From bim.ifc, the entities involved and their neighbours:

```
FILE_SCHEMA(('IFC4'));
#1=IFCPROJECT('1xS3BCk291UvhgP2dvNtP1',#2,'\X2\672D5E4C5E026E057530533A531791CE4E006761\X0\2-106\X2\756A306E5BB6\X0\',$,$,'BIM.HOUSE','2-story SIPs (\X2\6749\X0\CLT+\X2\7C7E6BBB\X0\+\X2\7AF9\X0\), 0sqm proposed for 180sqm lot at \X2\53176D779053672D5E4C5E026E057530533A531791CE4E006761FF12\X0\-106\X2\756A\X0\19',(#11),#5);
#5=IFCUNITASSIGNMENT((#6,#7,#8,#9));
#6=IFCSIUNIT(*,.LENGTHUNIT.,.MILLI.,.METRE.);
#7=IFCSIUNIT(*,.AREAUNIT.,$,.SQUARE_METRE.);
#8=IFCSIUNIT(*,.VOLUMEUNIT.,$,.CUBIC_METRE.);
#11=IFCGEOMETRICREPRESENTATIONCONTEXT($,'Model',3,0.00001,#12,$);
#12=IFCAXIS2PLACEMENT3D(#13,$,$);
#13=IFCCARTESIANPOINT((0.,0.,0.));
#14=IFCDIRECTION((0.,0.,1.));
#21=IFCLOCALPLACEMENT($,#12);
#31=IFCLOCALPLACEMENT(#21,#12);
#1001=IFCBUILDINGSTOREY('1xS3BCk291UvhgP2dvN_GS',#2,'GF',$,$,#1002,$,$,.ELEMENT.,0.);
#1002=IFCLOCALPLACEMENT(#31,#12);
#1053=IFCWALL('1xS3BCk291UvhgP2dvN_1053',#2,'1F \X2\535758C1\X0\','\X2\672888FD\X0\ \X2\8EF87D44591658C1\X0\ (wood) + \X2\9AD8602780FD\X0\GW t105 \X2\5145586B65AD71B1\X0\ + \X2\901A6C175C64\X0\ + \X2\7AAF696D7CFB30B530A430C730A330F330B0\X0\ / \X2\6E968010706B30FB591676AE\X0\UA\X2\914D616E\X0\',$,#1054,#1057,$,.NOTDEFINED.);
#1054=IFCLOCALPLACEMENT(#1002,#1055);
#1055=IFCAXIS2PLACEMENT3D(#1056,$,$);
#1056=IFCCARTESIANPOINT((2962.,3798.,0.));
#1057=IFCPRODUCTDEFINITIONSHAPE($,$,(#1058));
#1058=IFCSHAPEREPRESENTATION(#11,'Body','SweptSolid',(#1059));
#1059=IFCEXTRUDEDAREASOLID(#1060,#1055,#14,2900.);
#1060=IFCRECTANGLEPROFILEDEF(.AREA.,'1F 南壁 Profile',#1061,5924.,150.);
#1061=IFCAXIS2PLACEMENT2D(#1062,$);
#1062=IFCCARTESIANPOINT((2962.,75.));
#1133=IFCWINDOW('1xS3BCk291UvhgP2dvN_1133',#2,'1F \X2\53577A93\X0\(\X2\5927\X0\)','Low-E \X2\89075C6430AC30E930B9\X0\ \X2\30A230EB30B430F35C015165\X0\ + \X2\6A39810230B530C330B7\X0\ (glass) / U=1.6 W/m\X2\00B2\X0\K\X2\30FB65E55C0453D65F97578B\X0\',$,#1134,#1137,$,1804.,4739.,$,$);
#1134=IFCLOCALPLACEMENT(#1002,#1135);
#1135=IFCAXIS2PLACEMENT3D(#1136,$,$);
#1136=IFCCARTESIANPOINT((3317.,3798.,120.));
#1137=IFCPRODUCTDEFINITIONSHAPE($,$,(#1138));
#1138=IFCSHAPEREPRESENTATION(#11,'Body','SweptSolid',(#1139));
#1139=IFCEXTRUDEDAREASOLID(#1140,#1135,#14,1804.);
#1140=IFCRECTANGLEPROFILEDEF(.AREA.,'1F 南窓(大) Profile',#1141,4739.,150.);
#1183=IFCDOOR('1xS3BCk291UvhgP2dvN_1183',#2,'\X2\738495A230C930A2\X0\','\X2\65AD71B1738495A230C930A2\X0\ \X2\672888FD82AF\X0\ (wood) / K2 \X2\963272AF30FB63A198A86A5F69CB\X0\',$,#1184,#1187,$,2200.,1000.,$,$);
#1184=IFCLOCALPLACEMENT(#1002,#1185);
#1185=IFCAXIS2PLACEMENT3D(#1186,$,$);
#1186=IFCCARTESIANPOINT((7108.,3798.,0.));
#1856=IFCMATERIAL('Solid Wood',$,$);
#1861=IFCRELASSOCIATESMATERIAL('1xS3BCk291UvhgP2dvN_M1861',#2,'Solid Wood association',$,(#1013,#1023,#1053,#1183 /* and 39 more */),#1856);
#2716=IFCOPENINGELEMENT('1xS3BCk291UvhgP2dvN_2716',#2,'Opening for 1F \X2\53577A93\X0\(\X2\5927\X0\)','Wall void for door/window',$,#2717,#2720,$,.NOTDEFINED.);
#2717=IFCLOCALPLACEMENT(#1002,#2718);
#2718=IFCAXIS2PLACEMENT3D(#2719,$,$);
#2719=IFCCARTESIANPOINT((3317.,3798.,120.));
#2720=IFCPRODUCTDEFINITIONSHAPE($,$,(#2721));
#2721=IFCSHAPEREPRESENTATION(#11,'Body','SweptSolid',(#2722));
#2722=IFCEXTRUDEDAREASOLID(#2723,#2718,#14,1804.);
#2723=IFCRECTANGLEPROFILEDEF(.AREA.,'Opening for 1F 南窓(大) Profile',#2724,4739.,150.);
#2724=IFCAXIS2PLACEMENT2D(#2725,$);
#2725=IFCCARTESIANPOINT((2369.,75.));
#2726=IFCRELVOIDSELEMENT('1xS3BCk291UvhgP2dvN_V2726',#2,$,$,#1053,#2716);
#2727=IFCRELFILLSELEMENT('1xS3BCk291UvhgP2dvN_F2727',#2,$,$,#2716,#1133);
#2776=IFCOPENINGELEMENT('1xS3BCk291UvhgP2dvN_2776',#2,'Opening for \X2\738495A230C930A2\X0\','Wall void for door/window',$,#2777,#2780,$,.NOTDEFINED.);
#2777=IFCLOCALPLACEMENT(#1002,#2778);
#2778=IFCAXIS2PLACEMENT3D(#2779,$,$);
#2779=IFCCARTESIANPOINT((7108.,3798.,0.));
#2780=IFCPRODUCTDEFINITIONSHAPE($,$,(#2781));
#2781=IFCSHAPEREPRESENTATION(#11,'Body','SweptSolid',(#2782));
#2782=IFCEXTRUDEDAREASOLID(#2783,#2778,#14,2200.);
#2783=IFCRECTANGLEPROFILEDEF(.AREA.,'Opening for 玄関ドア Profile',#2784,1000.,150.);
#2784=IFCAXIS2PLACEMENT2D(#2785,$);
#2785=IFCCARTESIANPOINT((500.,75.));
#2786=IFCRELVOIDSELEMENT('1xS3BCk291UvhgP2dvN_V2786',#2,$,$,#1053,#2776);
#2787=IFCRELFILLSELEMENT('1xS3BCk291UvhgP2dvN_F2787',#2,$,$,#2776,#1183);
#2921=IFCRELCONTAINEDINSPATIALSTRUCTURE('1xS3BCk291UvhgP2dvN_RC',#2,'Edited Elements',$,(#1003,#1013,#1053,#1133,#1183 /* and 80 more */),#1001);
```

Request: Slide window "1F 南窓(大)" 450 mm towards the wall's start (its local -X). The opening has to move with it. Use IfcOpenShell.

```python
import ifcopenshell
import ifcopenshell.api.geometry
import ifcopenshell.util.placement

model = ifcopenshell.open("bim.ifc")

window = model.by_id(1133)
opening = window.FillsVoids[0].RelatingOpeningElement
wall = opening.VoidsElements[0].RelatingBuildingElement

wall_matrix = ifcopenshell.util.placement.get_local_placement(wall.ObjectPlacement)
shift = wall_matrix[:3, 0] * -450.0
before = ifcopenshell.util.placement.get_local_placement(window.ObjectPlacement)[:3, 3].copy()

# The window is not placed relative to its opening, so move both.
for product in (opening, window):
    matrix = ifcopenshell.util.placement.get_local_placement(product.ObjectPlacement)
    matrix[:3, 3] += shift
    ifcopenshell.api.geometry.edit_object_placement(model, product=product, matrix=matrix, is_si=False)

after = ifcopenshell.util.placement.get_local_placement(window.ObjectPlacement)[:3, 3]
print("window moved by", (after - before).round(3) + 0.0)

model.write("bim_v2.ifc")
```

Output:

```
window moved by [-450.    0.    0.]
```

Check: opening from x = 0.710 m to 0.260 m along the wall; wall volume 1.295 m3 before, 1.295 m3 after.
